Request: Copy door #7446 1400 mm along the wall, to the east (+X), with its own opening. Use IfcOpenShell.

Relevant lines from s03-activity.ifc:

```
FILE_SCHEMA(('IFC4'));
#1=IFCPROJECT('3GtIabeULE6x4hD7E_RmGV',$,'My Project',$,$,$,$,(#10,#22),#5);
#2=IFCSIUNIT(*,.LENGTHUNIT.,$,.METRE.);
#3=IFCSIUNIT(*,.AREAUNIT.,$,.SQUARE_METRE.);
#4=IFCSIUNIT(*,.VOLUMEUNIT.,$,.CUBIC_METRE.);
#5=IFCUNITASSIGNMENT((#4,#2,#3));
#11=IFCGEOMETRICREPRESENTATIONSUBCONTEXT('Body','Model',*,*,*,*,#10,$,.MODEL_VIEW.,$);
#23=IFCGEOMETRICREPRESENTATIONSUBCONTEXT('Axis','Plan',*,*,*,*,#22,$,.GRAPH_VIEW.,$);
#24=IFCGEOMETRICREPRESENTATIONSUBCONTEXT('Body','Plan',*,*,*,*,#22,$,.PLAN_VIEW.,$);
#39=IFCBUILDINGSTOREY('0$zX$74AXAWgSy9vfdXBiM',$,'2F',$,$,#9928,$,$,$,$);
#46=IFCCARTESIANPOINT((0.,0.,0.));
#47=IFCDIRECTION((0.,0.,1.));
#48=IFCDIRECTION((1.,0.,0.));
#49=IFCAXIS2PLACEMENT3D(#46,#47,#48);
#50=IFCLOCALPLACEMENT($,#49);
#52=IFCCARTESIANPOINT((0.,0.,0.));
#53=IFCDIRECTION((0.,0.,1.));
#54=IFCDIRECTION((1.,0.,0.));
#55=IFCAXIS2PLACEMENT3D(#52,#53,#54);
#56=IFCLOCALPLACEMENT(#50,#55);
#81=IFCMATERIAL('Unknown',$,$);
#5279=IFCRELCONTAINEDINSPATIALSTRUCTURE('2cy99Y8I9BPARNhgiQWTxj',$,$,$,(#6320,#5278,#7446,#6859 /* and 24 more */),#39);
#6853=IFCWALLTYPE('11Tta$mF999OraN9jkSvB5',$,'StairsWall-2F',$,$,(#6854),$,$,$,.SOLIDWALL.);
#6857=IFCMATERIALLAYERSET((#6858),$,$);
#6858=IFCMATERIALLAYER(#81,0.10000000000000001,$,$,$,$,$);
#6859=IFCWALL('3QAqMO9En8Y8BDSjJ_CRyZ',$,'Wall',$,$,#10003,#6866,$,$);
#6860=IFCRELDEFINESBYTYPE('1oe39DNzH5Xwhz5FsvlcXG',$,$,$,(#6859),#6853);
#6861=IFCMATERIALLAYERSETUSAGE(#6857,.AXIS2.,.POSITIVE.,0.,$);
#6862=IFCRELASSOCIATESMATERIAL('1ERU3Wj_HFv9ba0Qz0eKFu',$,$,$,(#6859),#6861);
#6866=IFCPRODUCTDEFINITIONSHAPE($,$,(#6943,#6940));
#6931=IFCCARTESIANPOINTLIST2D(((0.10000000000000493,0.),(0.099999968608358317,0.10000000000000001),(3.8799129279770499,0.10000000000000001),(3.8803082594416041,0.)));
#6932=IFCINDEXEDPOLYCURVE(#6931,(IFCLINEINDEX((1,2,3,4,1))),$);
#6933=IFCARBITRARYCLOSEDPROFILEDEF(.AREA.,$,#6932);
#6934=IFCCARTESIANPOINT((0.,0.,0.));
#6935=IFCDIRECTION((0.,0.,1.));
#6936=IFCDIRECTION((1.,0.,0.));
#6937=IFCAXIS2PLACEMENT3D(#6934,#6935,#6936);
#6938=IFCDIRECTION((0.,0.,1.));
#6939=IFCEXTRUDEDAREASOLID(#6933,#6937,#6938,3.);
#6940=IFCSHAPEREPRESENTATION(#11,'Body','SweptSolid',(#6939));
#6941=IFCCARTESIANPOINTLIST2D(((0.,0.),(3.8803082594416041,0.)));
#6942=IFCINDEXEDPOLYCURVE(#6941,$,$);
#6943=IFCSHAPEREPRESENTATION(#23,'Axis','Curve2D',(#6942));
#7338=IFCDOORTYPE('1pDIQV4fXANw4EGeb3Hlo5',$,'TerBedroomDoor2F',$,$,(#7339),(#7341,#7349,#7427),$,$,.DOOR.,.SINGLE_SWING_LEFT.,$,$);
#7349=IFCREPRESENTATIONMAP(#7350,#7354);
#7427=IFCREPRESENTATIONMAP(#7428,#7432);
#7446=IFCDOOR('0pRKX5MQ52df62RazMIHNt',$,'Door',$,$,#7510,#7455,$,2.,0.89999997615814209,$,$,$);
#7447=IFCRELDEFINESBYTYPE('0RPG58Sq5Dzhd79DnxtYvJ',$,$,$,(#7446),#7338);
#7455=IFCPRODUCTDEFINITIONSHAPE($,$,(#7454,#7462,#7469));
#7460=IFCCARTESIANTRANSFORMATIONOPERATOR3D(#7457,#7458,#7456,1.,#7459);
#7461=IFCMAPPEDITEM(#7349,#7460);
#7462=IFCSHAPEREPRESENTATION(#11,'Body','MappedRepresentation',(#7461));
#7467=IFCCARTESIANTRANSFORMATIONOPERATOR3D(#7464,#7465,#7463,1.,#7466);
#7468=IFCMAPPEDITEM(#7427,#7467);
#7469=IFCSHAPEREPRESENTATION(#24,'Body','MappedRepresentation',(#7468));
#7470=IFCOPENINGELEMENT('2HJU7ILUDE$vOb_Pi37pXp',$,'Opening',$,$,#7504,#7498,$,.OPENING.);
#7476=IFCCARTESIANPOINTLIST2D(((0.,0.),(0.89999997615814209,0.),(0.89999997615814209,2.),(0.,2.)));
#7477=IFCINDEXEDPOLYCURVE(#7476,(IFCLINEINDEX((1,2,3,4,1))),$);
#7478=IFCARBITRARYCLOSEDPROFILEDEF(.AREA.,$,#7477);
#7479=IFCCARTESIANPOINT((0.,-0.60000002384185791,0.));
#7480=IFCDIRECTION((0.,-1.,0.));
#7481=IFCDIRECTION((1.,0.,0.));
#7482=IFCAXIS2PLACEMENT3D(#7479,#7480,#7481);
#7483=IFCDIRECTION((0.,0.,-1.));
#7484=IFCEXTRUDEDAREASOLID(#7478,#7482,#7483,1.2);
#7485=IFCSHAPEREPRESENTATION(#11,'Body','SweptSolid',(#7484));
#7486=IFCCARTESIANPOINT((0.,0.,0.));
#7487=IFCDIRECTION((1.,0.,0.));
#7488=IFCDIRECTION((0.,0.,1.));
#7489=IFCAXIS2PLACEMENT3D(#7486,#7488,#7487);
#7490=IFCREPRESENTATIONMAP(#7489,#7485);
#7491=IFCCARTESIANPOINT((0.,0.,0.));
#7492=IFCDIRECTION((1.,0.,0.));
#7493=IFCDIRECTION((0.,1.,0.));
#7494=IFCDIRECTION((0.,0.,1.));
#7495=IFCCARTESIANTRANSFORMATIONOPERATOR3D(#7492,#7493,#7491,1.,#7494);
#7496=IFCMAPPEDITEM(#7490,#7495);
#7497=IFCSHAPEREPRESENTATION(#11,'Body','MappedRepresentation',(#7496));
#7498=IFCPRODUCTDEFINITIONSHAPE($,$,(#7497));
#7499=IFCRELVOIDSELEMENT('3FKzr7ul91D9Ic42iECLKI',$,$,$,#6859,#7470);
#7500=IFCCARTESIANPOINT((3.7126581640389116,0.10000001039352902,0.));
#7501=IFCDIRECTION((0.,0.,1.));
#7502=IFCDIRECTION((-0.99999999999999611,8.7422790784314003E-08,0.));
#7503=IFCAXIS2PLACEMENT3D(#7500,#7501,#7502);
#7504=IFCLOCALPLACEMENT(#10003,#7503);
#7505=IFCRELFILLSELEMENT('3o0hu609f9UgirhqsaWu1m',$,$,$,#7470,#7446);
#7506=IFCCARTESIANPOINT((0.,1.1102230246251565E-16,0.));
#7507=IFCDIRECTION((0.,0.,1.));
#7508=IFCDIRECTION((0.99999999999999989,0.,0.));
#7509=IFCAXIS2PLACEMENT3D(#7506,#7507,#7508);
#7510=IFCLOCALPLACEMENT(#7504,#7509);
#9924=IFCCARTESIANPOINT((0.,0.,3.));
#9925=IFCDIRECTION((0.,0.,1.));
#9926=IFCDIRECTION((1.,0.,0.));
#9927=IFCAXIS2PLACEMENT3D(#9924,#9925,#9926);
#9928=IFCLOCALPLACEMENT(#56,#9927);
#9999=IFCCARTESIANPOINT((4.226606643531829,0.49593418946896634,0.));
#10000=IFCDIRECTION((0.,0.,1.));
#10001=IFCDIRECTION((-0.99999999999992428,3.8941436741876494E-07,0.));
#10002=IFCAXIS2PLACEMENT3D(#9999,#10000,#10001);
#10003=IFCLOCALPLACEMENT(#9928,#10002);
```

```python
import ifcopenshell
import ifcopenshell.api.feature
import ifcopenshell.api.geometry
import ifcopenshell.api.root
import ifcopenshell.geom
import ifcopenshell.util.element
import ifcopenshell.util.placement
import ifcopenshell.util.shape

model = ifcopenshell.open("s03-activity.ifc")
settings = ifcopenshell.geom.settings()


def volume(element):
    """Net volume in cubic metres, openings subtracted."""
    shape = ifcopenshell.geom.create_shape(settings, element)
    return ifcopenshell.util.shape.get_volume(shape.geometry)


door = model.by_guid("0pRKX5MQ52df62RazMIHNt")
opening = door.FillsVoids[0].RelatingOpeningElement
wall = opening.VoidsElements[0].RelatingBuildingElement
before = volume(wall)
shift = ifcopenshell.util.placement.get_local_placement(wall.ObjectPlacement)[:3, 0] * -1.4

# copy_class copies the void relationship, type, container and properties, but no geometry.
new_opening = ifcopenshell.api.root.copy_class(model, product=opening)
new_opening.Representation = ifcopenshell.util.element.copy_deep(
    model, opening.Representation, exclude=["IfcGeometricRepresentationContext", "IfcRepresentationMap"]
)
new_door = ifcopenshell.api.root.copy_class(model, product=door)
new_door.Representation = ifcopenshell.util.element.copy_deep(
    model, door.Representation, exclude=["IfcGeometricRepresentationContext", "IfcRepresentationMap"]
)
ifcopenshell.api.feature.add_filling(model, opening=new_opening, element=new_door)

for old, new in ((opening, new_opening), (door, new_door)):
    matrix = ifcopenshell.util.placement.get_local_placement(old.ObjectPlacement)
    matrix[:3, 3] += shift
    ifcopenshell.api.geometry.edit_object_placement(model, product=new, matrix=matrix, is_si=False)

after = volume(wall)

print(f"wall volume {before:.3f} -> {after:.3f} m3")

model.write("s03-activity_edited.ifc")
```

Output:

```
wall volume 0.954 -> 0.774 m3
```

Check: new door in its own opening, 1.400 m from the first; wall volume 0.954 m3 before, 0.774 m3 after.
